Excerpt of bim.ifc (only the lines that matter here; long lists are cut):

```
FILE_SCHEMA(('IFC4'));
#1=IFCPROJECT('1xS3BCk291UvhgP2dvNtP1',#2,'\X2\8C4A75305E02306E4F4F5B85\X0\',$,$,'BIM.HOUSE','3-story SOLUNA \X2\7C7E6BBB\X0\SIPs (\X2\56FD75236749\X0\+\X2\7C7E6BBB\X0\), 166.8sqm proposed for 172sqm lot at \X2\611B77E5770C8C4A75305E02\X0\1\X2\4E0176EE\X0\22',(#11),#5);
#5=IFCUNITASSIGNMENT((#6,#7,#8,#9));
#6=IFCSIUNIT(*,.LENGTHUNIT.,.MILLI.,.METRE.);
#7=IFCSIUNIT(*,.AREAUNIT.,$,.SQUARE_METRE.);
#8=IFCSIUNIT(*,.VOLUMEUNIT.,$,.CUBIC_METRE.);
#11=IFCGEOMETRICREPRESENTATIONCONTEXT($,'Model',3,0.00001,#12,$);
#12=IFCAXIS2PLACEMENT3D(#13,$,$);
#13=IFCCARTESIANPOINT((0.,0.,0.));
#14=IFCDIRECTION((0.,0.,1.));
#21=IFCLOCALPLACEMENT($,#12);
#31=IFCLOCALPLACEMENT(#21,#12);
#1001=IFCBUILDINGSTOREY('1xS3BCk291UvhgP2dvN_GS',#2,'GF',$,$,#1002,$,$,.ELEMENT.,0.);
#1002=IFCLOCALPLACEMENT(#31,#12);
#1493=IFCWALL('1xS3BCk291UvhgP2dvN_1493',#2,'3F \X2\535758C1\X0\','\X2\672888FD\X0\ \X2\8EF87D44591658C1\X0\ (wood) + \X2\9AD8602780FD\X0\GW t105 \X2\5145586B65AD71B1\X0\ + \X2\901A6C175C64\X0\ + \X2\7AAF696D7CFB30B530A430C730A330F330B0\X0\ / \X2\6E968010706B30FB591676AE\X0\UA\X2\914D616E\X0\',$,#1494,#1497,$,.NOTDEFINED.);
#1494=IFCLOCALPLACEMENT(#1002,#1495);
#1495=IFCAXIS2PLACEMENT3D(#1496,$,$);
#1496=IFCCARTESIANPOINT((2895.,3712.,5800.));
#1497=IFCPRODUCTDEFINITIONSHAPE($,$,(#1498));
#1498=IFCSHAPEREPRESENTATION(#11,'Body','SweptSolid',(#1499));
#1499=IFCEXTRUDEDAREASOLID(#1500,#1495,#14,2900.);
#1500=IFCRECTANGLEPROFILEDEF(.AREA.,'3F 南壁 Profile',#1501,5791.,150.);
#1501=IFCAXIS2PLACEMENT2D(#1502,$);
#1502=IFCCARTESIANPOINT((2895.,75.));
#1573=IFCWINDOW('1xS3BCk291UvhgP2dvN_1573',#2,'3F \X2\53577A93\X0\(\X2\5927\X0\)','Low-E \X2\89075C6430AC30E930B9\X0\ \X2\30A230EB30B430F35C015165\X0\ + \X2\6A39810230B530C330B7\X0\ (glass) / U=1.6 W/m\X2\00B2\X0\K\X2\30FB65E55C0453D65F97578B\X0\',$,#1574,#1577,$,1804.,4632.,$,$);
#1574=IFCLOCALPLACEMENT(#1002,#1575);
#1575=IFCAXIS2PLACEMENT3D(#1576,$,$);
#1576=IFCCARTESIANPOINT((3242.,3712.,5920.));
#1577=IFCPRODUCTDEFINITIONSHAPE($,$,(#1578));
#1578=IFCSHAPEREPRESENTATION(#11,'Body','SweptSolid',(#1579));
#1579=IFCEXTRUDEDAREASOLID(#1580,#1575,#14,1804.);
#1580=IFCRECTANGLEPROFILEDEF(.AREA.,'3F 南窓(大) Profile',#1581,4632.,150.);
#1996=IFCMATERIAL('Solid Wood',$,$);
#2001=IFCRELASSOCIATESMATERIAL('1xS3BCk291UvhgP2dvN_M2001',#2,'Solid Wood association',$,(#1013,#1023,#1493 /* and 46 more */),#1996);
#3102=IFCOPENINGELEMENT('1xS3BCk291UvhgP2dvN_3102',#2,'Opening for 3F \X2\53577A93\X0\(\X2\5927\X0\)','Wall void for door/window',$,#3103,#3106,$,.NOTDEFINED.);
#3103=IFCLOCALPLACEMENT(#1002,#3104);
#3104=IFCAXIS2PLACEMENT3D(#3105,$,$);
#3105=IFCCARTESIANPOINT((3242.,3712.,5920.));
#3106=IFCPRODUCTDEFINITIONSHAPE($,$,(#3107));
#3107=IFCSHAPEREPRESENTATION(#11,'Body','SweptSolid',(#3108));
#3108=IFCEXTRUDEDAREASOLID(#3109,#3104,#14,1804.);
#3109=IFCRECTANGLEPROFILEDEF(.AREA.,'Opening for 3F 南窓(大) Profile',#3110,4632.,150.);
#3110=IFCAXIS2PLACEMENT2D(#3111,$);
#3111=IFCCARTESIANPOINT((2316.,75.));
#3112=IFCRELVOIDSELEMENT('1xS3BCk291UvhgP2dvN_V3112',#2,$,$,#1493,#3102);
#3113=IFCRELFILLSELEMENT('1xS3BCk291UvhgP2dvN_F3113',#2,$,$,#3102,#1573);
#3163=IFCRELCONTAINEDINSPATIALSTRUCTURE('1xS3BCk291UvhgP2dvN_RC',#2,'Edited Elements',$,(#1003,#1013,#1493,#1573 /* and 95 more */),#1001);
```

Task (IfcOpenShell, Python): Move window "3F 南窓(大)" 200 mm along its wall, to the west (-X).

```python
import ifcopenshell
import ifcopenshell.api.geometry
import ifcopenshell.util.placement
import ifcopenshell.util.unit

model = ifcopenshell.open("bim.ifc")
unit_scale = ifcopenshell.util.unit.calculate_unit_scale(model)

window = model.by_guid("1xS3BCk291UvhgP2dvN_1573")
opening = window.FillsVoids[0].RelatingOpeningElement
wall = opening.VoidsElements[0].RelatingBuildingElement

wall_matrix = ifcopenshell.util.placement.get_local_placement(wall.ObjectPlacement)
shift = wall_matrix[:3, 0] * -0.2 / unit_scale
before = ifcopenshell.util.placement.get_local_placement(window.ObjectPlacement)[:3, 3].copy()

# The window is not placed relative to its opening, so move both.
for product in (opening, window):
    matrix = ifcopenshell.util.placement.get_local_placement(product.ObjectPlacement)
    matrix[:3, 3] += shift
    ifcopenshell.api.geometry.edit_object_placement(model, product=product, matrix=matrix, is_si=False)

after = ifcopenshell.util.placement.get_local_placement(window.ObjectPlacement)[:3, 3]
print("window moved by", (after - before).round(3) + 0.0)

model.write("bim_rev.ifc")
```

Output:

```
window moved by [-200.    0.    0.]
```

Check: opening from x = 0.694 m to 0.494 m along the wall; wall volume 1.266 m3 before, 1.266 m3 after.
